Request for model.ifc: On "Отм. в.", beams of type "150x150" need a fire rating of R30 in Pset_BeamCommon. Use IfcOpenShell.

First a look at what the model holds.

```python
import ifcopenshell
import ifcopenshell.util.element

model = ifcopenshell.open("model.ifc")
print(model.schema)
storey = next(s for s in model.by_type("IfcBuildingStorey") if s.Name == "Отм. в.")
beams = [e for e in ifcopenshell.util.element.get_decomposition(storey) if e.is_a("IfcBeam")]
seen = {}
for e in beams:
    element_type = ifcopenshell.util.element.get_type(e)
    key = (element_type.Name if element_type != e and element_type else None, ifcopenshell.util.element.get_pset(e, "Pset_BeamCommon", "FireRating"))
    seen[key] = seen.get(key, 0) + 1
for (name, value), count in sorted(seen.items(), key=str):
    print(count, "x", name, "|", value)
```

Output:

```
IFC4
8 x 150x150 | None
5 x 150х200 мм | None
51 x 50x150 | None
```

```python
import ifcopenshell
import ifcopenshell.api.pset
import ifcopenshell.util.element

model = ifcopenshell.open("model.ifc")

storey = next(s for s in model.by_type("IfcBuildingStorey") if s.Name == "Отм. в.")
beams = [e for e in ifcopenshell.util.element.get_decomposition(storey) if e.is_a("IfcBeam")]

count = 0
for e in beams:
    element_type = ifcopenshell.util.element.get_type(e)
    if element_type in (None, e) or element_type.Name != "150x150":
        continue
    # add_pset returns the element's existing set when there is one.
    pset = ifcopenshell.api.pset.add_pset(model, product=e, name="Pset_BeamCommon")
    ifcopenshell.api.pset.edit_pset(model, pset=pset, properties={"FireRating": "R30"})
    count += 1

print(count, "beams updated")

model.write("model-out.ifc")
```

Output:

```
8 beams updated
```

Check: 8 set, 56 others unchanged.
